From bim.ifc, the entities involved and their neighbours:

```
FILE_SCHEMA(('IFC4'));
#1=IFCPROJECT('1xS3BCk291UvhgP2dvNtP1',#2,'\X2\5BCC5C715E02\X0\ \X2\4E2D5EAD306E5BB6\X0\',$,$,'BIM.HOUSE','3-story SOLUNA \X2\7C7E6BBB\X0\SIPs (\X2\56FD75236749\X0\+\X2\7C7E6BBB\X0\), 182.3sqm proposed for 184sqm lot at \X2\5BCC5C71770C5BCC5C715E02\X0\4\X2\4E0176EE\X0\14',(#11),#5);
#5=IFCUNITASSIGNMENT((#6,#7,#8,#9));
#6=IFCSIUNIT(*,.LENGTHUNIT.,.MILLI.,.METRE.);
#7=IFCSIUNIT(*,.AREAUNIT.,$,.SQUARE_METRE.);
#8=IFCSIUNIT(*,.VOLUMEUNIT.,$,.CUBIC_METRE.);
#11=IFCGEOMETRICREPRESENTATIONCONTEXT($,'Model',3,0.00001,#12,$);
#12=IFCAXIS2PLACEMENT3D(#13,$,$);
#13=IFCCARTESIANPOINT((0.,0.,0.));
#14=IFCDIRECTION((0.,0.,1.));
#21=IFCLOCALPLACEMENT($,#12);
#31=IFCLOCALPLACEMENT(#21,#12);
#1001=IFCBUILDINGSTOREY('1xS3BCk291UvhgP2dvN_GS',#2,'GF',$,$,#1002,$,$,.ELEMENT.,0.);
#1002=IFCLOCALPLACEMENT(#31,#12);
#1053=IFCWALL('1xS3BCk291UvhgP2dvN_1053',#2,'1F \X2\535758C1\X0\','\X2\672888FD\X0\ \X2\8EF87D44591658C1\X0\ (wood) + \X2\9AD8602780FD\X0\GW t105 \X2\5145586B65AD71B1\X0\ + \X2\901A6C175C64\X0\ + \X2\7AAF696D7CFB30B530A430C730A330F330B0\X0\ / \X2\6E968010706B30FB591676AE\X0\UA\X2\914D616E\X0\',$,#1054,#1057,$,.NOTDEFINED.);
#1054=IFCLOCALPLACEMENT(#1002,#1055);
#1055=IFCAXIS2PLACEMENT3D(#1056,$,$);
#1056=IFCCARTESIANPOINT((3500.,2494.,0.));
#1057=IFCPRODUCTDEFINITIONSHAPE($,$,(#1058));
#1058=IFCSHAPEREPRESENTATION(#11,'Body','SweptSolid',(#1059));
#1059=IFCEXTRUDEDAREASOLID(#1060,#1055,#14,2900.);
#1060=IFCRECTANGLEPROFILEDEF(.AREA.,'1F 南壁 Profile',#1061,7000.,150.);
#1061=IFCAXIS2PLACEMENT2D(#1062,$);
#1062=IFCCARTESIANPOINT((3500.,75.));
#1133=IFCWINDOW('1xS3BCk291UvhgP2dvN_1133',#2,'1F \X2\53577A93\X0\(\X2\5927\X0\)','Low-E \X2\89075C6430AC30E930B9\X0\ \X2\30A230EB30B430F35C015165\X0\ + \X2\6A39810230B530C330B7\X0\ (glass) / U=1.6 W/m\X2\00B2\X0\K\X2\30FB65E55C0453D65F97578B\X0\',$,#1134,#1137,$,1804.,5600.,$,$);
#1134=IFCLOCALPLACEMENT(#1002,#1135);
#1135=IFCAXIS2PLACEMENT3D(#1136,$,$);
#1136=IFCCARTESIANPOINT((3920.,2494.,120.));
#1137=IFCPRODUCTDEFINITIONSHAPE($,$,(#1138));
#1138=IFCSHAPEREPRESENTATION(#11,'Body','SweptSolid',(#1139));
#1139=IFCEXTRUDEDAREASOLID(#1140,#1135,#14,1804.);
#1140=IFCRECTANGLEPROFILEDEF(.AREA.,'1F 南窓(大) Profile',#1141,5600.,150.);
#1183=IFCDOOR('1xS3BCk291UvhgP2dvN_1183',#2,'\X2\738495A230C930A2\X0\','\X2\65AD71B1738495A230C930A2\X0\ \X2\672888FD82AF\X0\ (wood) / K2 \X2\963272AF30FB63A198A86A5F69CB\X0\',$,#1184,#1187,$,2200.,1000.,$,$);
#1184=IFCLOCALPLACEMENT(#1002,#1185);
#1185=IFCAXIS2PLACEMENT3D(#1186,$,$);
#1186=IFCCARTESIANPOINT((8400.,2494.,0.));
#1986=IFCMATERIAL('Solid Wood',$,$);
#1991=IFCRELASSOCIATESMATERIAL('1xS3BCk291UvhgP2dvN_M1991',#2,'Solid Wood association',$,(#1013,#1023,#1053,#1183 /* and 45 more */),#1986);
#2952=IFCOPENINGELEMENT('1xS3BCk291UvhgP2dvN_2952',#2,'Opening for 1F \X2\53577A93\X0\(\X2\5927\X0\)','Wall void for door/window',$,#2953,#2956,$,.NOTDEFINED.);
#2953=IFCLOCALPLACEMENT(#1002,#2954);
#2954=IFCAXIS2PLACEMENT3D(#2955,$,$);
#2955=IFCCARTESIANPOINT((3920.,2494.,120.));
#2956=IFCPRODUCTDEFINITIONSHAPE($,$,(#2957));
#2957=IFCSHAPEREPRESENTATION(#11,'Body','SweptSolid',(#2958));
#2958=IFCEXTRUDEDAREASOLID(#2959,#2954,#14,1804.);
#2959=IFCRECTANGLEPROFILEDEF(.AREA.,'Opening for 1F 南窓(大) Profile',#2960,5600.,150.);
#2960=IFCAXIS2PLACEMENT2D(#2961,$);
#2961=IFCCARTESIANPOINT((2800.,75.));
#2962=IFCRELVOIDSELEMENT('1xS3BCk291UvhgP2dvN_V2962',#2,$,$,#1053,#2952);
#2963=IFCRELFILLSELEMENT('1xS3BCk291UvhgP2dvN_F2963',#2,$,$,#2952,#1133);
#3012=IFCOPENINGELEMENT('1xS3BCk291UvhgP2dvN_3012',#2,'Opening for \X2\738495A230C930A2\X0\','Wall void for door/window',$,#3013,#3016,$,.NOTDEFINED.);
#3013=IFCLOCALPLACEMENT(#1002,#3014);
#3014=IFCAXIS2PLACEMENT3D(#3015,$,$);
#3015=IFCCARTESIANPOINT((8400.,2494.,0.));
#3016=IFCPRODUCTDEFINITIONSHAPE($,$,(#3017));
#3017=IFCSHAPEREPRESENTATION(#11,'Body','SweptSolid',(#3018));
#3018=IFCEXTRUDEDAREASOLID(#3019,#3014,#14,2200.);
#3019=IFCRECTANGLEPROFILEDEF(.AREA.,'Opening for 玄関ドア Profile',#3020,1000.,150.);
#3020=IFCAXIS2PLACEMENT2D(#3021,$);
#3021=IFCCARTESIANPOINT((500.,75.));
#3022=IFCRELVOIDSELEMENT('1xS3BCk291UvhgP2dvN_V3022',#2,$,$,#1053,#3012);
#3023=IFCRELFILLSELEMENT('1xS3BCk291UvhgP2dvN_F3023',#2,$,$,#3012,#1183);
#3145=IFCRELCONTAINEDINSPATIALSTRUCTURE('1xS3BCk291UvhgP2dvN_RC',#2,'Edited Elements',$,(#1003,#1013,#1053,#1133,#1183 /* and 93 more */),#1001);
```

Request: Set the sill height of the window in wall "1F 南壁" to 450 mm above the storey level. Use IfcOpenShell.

```python
import numpy as np
import ifcopenshell
import ifcopenshell.api.geometry
import ifcopenshell.geom
import ifcopenshell.util.element
import ifcopenshell.util.placement
import ifcopenshell.util.shape
import ifcopenshell.util.unit

model = ifcopenshell.open("bim.ifc")
unit_scale = ifcopenshell.util.unit.calculate_unit_scale(model)

window = model.by_guid("1xS3BCk291UvhgP2dvN_1133")
opening = window.FillsVoids[0].RelatingOpeningElement
storey = ifcopenshell.util.element.get_container(window, ifc_class="IfcBuildingStorey")
level = ifcopenshell.util.placement.get_local_placement(storey.ObjectPlacement)[2, 3]

# The opening's origin need not be at the sill, so measure its lowest point.
shape = ifcopenshell.geom.create_shape(ifcopenshell.geom.settings(), opening)
bottom = ifcopenshell.util.shape.get_shape_bottom_elevation(shape, shape.geometry) / unit_scale
dz = level + 450.0 - bottom

shift = np.array([0.0, 0.0, dz])
# The window is not placed relative to its opening, so move both.
for product in (opening, window):
    matrix = ifcopenshell.util.placement.get_local_placement(product.ObjectPlacement)
    matrix[:3, 3] += shift
    ifcopenshell.api.geometry.edit_object_placement(model, product=product, matrix=matrix, is_si=False)

print(f"moved by {dz * unit_scale:+.3f} m")

model.write("bim-out.ifc")
```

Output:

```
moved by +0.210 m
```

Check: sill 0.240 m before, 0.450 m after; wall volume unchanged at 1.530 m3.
